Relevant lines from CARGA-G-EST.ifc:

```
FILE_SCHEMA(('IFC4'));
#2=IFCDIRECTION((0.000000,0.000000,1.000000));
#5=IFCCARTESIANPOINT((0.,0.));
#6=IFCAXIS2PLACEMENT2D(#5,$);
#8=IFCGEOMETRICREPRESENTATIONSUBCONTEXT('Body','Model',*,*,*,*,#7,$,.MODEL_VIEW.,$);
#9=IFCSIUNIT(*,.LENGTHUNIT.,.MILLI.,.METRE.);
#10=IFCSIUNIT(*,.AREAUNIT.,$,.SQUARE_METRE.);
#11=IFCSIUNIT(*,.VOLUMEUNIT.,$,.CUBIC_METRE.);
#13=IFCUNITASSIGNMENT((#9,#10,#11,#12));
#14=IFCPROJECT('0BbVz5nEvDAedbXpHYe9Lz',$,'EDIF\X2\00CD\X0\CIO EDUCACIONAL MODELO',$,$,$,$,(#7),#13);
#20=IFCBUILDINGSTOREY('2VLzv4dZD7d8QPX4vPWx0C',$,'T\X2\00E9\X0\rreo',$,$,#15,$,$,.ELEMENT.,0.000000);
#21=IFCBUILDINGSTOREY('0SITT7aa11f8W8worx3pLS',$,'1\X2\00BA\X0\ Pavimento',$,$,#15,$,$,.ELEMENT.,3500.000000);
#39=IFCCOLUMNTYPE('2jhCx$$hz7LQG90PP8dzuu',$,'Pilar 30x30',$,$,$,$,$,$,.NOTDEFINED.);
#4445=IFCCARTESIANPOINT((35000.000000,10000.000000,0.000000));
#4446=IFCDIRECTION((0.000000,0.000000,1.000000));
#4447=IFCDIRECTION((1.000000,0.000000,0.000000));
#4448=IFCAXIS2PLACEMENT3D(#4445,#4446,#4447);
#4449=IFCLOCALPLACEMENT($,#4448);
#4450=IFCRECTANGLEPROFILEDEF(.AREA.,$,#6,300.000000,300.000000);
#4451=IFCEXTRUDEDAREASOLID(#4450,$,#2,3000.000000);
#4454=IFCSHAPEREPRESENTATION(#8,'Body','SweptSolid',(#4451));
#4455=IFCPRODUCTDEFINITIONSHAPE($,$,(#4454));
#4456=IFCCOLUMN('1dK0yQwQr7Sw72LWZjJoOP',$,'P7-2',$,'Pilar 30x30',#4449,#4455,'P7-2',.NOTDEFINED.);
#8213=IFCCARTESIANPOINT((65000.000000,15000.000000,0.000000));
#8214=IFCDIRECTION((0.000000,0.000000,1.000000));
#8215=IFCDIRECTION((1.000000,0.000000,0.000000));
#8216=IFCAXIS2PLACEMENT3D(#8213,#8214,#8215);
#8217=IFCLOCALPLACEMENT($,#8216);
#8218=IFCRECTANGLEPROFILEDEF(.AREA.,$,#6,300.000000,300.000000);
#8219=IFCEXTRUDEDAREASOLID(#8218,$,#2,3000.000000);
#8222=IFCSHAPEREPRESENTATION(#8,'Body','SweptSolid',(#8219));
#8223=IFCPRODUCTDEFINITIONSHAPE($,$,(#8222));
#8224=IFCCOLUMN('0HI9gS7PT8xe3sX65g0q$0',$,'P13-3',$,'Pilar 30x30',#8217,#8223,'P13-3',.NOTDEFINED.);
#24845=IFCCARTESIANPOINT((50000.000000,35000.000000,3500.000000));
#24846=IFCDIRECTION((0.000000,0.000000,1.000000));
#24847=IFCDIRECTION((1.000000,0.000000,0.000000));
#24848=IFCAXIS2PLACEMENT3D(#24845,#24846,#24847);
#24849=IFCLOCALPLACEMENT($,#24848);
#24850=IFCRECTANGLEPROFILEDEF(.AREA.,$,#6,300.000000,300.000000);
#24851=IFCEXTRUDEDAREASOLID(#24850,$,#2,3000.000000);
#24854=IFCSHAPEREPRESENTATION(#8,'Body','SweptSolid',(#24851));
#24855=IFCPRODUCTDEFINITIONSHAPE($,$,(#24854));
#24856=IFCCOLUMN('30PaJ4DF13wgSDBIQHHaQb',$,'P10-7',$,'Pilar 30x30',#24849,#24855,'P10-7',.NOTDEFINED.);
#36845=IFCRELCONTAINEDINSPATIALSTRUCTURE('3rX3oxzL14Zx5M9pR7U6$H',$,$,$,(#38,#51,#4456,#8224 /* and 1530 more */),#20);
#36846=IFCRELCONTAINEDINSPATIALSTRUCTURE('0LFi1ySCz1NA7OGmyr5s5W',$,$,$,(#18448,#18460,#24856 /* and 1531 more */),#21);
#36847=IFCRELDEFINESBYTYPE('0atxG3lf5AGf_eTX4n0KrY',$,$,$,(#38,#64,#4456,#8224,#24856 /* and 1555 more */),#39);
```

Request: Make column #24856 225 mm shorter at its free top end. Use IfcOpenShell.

```python
import ifcopenshell
import ifcopenshell.util.representation

model = ifcopenshell.open("CARGA-G-EST.ifc")

member = model.by_guid("30PaJ4DF13wgSDBIQHHaQb")
change = -225.0

# The extrusion runs towards the end named, so only its depth changes.
body = ifcopenshell.util.representation.get_representation(member, "Model", "Body")
solid = body.Items[0]
old_length = solid.Depth
solid.Depth += change

print(f"length {old_length:g} -> {solid.Depth:g}")

model.write("CARGA-G-EST_edited.ifc")
```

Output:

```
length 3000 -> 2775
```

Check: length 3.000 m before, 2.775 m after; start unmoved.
